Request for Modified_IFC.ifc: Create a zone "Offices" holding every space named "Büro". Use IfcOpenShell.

First a look at what the model holds.

```python
import ifcopenshell

model = ifcopenshell.open("Modified_IFC.ifc")
print(model.schema)
seen = {}
for space in model.by_type("IfcSpace"):
    seen[space.LongName] = seen.get(space.LongName, 0) + 1
for name, count in sorted(seen.items(), key=str):
    print(count, "x", name)
print("zones:", [z.Name for z in model.by_type("IfcZone")][:20])
```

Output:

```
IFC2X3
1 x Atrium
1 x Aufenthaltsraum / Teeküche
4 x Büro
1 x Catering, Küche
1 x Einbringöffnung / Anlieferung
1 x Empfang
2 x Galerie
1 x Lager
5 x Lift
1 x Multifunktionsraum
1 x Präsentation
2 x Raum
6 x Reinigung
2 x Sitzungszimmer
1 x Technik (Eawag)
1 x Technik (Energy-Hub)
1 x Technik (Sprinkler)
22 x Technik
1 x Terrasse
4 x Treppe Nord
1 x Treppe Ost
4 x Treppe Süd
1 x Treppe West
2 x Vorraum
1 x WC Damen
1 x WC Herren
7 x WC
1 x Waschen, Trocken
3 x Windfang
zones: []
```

```python
import ifcopenshell
import ifcopenshell.api.group
import ifcopenshell.api.root

model = ifcopenshell.open("Modified_IFC.ifc")

names = {"Büro"}
spaces = [s for s in model.by_type("IfcSpace") if s.LongName in names]

zone = ifcopenshell.api.root.create_entity(model, ifc_class="IfcZone", name="Offices")
ifcopenshell.api.group.assign_group(model, products=spaces, group=zone)
print(len(spaces), "spaces in", zone.Name)

model.write("Modified_IFC_edited.ifc")
```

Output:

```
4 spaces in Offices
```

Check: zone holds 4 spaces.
